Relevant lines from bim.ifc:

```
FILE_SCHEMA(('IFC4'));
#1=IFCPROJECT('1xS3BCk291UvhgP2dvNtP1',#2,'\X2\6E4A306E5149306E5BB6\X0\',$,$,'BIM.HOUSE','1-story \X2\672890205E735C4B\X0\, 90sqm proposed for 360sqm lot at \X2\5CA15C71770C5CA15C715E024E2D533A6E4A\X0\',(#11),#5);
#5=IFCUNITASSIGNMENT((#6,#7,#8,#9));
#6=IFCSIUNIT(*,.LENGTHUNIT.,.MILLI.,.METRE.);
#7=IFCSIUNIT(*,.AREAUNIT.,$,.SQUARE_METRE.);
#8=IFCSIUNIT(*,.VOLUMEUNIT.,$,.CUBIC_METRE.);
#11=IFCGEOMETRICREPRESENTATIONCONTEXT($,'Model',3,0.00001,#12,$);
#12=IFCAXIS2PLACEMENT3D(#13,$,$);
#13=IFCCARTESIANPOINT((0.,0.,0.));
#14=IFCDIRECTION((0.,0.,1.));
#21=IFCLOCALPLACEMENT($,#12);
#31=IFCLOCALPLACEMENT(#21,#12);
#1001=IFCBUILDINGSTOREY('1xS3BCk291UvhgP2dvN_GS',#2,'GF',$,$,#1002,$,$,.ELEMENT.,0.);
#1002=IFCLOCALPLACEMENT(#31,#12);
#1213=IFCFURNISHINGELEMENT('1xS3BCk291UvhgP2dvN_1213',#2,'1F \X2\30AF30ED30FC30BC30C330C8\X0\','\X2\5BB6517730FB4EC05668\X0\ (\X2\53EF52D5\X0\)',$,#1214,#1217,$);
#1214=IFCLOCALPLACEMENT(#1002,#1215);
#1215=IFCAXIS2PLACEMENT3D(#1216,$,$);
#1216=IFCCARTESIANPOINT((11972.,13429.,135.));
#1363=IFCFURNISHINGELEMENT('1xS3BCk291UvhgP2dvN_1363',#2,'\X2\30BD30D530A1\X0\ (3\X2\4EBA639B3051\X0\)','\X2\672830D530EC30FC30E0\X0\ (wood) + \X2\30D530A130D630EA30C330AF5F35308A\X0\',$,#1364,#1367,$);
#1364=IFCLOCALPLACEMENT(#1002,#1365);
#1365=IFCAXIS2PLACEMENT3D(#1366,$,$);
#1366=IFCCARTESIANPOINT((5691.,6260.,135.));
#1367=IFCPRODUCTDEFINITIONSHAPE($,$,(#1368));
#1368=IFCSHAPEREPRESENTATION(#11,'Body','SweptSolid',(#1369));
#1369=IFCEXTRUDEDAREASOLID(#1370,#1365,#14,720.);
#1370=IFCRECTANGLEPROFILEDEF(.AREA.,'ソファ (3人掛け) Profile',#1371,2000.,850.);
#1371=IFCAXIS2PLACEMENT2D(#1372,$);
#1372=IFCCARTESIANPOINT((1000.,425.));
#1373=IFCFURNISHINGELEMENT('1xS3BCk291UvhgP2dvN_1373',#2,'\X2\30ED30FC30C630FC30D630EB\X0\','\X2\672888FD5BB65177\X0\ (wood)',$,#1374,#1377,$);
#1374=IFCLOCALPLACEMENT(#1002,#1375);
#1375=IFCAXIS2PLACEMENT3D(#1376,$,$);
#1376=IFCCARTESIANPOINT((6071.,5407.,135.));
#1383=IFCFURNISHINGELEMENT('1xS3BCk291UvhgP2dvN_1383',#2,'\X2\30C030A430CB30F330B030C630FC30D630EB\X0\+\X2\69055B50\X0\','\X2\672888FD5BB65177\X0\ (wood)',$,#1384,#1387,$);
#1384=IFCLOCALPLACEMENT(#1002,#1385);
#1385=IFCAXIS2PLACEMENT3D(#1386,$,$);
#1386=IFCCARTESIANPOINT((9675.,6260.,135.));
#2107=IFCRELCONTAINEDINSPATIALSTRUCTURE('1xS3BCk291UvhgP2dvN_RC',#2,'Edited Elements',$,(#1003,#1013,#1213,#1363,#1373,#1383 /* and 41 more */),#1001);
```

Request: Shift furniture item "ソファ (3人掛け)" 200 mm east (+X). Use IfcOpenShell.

```python
import ifcopenshell
import ifcopenshell.api.geometry
import ifcopenshell.util.placement
import ifcopenshell.util.unit

model = ifcopenshell.open("bim.ifc")
unit_scale = ifcopenshell.util.unit.calculate_unit_scale(model)

item = model.by_guid("1xS3BCk291UvhgP2dvN_1363")
matrix = ifcopenshell.util.placement.get_local_placement(item.ObjectPlacement)
matrix[0, 3] += 0.2 / unit_scale
ifcopenshell.api.geometry.edit_object_placement(model, product=item, matrix=matrix, is_si=False)

print(ifcopenshell.util.placement.get_local_placement(item.ObjectPlacement).round(3) + 0.0)

model.write("bim_v2.ifc")
```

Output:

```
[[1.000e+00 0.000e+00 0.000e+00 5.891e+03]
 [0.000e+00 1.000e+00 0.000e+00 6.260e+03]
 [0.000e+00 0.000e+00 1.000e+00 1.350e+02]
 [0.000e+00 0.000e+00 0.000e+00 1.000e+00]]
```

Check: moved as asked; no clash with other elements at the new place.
